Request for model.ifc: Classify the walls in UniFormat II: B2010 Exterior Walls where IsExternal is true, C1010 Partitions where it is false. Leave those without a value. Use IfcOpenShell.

First a look at what the model holds.

```python
import ifcopenshell
import ifcopenshell.util.element

model = ifcopenshell.open("model.ifc")
print(model.schema)
print("classifications:", [c.Name for c in model.by_type("IfcClassification")])
values = [ifcopenshell.util.element.get_pset(e, "Pset_WallCommon", "IsExternal") for e in model.by_type("IfcWall")]
for value in (True, False, None):
    print("IsExternal", value, values.count(value))
```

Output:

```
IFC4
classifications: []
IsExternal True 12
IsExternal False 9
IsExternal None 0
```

```python
import ifcopenshell
import ifcopenshell.api.classification
import ifcopenshell.util.element

model = ifcopenshell.open("model.ifc")

system = ifcopenshell.api.classification.add_classification(model, classification="UniFormat II")

walls = model.by_type("IfcWall")
external = {e: ifcopenshell.util.element.get_pset(e, "Pset_WallCommon", "IsExternal") for e in walls}
for flag, code, name in ((True, "B2010", "Exterior Walls"), (False, "C1010", "Partitions")):
    products = [e for e in walls if external[e] is flag]
    ifcopenshell.api.classification.add_reference(
        model, products=products, classification=system, identification=code, name=name
    )
    print(code, len(products))

model.write("model_updated.ifc")
```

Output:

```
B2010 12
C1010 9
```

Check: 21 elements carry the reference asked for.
